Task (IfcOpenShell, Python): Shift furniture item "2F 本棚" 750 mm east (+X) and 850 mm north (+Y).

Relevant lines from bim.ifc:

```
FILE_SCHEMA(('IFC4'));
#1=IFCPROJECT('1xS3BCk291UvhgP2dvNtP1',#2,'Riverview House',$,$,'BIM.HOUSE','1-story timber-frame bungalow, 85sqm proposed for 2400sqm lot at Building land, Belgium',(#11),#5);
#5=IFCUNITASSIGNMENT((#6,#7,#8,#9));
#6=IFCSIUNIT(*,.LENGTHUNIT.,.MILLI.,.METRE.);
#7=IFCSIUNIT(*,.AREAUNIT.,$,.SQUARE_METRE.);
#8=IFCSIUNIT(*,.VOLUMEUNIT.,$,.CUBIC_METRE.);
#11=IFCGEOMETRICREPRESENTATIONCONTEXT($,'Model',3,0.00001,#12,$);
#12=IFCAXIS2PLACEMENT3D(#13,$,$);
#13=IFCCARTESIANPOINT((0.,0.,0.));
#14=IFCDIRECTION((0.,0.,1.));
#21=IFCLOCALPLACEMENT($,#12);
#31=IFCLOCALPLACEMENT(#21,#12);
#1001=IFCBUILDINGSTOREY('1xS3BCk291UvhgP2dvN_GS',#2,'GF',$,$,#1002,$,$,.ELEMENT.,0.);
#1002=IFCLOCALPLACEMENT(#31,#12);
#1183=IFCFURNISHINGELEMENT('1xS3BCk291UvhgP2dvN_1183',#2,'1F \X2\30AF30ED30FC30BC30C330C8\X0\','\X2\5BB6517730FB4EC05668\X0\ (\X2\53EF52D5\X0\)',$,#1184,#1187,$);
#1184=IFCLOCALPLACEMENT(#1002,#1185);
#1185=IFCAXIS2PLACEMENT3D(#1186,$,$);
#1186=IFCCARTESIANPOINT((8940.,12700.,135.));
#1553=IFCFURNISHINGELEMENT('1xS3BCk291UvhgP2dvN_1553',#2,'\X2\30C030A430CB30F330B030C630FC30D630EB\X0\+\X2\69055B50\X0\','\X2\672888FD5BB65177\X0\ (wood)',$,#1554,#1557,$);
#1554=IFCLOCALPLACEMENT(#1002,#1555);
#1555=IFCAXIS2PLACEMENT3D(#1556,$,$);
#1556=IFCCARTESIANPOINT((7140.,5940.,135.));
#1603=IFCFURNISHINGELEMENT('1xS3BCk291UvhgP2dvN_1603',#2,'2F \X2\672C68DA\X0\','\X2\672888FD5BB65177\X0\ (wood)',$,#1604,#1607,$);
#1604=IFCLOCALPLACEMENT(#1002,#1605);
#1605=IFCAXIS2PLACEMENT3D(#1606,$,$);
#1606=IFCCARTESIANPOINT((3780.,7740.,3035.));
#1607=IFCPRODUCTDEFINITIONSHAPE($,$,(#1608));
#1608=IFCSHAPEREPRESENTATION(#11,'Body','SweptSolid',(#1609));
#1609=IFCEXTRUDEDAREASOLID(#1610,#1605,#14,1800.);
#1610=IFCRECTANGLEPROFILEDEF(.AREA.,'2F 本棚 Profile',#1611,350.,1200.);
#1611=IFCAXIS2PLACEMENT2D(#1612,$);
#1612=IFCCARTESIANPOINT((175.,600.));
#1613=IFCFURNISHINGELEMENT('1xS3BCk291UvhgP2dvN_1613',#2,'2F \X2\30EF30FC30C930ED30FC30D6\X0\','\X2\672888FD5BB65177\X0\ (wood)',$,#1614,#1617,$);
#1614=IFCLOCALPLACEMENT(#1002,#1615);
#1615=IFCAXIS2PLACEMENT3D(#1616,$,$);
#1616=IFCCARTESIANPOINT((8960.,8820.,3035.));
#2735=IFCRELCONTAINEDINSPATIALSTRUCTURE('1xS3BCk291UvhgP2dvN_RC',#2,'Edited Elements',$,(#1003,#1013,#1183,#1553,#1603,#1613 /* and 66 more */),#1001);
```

```python
import ifcopenshell
import ifcopenshell.api.geometry
import ifcopenshell.util.placement
import ifcopenshell.util.unit

model = ifcopenshell.open("bim.ifc")
unit_scale = ifcopenshell.util.unit.calculate_unit_scale(model)

item = model.by_guid("1xS3BCk291UvhgP2dvN_1603")
matrix = ifcopenshell.util.placement.get_local_placement(item.ObjectPlacement)
matrix[0, 3] += 0.75 / unit_scale
matrix[1, 3] += 0.85 / unit_scale
ifcopenshell.api.geometry.edit_object_placement(model, product=item, matrix=matrix, is_si=False)

print(ifcopenshell.util.placement.get_local_placement(item.ObjectPlacement).round(3) + 0.0)

model.write("bim_v2.ifc")
```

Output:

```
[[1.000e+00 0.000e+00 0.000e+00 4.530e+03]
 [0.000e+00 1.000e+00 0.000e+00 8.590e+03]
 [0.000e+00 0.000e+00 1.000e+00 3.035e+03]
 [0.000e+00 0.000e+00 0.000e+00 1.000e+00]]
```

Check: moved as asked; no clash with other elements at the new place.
